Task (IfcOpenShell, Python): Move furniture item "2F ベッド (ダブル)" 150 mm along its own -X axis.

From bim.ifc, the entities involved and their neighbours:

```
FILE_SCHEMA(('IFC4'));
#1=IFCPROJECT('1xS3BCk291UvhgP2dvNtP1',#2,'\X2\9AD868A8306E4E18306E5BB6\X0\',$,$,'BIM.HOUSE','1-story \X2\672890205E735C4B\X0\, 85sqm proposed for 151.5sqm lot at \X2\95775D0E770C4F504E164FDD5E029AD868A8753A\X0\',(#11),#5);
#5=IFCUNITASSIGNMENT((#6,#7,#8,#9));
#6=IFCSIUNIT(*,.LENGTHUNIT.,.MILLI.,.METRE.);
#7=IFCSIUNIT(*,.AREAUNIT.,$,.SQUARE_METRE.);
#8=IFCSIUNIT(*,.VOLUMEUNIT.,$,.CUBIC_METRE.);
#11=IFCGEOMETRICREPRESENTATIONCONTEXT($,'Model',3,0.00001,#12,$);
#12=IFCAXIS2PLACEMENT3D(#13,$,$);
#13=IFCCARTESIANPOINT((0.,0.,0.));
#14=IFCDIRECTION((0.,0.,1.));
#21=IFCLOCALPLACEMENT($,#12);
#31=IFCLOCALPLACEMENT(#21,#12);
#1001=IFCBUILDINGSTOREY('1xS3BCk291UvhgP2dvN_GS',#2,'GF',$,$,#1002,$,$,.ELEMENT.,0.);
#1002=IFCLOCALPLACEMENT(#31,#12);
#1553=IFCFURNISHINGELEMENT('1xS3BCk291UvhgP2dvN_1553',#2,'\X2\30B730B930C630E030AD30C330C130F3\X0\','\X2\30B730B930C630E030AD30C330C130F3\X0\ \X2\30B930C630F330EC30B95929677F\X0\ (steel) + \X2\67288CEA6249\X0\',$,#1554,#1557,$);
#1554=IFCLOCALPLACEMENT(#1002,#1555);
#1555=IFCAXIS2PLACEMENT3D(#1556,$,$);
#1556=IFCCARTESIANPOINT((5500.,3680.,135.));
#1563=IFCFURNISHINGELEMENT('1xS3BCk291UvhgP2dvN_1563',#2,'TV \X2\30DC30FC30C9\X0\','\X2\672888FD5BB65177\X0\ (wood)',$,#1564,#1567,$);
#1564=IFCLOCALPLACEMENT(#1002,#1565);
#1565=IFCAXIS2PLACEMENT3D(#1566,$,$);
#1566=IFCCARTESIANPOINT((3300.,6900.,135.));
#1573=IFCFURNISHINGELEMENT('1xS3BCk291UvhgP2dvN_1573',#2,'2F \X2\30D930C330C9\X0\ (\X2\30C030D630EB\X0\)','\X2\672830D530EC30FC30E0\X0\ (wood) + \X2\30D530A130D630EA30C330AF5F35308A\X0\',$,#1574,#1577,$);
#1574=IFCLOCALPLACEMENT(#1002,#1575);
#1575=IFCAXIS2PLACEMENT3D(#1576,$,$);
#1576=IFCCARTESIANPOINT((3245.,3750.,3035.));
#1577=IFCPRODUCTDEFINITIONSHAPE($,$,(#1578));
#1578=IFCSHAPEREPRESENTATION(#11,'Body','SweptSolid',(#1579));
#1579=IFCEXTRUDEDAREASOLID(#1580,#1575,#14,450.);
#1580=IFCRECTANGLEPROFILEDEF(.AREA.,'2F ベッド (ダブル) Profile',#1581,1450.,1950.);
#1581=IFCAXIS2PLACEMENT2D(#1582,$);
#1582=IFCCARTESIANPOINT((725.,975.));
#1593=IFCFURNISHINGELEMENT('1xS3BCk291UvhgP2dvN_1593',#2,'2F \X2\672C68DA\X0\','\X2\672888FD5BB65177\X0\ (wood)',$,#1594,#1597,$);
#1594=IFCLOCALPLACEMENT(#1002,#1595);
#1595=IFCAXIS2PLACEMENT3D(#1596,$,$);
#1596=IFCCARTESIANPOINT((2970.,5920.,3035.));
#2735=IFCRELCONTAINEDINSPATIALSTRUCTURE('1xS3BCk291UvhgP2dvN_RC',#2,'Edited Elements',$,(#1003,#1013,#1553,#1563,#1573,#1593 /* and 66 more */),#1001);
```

```python
import ifcopenshell
import ifcopenshell.api.geometry
import ifcopenshell.util.placement

model = ifcopenshell.open("bim.ifc")

item = model.by_guid("1xS3BCk291UvhgP2dvN_1573")
matrix = ifcopenshell.util.placement.get_local_placement(item.ObjectPlacement)
matrix[:3, 3] -= matrix[:3, 0] * 150.0
ifcopenshell.api.geometry.edit_object_placement(model, product=item, matrix=matrix, is_si=False)

print(ifcopenshell.util.placement.get_local_placement(item.ObjectPlacement).round(3) + 0.0)

model.write("bim_v2.ifc")
```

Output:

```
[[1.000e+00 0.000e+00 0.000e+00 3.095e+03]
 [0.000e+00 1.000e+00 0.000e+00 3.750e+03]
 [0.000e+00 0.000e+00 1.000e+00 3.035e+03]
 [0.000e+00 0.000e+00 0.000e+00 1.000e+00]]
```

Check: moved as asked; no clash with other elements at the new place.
